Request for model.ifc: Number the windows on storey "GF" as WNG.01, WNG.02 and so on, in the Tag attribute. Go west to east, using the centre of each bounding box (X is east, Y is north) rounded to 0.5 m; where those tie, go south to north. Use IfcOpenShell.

First a look at what the model holds.

```python
import ifcopenshell
import ifcopenshell.util.element
import ifcopenshell.util.placement

model = ifcopenshell.open("model.ifc")
print(model.schema)
storey = next(s for s in model.by_type("IfcBuildingStorey") if s.Name == "GF")
windows = [e for e in ifcopenshell.util.element.get_decomposition(storey) if e.is_a("IfcWindow")]
for e in sorted(windows, key=lambda e: e.id()):
    origin = ifcopenshell.util.placement.get_local_placement(e.ObjectPlacement)[:3, 3]
    print(e.id(), e.Tag, e.Name, origin.round(2) + 0.0, sep=" | ")
```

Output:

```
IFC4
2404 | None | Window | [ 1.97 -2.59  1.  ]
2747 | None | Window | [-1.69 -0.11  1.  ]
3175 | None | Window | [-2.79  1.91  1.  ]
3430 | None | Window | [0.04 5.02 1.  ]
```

```python
import ifcopenshell
import ifcopenshell.geom
import ifcopenshell.util.element
import ifcopenshell.util.shape

model = ifcopenshell.open("model.ifc")
settings = ifcopenshell.geom.settings()
settings.set("use-world-coords", True)


def centre(element):
    shape = ifcopenshell.geom.create_shape(settings, element)
    return ifcopenshell.util.shape.get_bbox_centroid(shape.geometry)


storey = next(s for s in model.by_type("IfcBuildingStorey") if s.Name == "GF")
windows = [e for e in ifcopenshell.util.element.get_decomposition(storey) if e.is_a("IfcWindow")]

# Insertion points can sit at a corner or the storey origin, so sort by the geometry (in metres).
centres = {e: centre(e) for e in windows}
windows.sort(key=lambda e: (round(centres[e][0] / 0.5), centres[e][1]))

for i, e in enumerate(windows, start=1):
    number = f"WNG.{i:02d}"
    e.Tag = number
    print(e.id(), number)

model.write("model_v2.ifc")
```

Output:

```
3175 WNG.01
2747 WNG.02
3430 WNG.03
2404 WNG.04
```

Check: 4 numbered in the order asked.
